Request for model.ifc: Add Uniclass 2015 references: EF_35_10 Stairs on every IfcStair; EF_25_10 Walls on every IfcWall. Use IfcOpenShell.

First a look at what the model holds.

```python
import ifcopenshell

model = ifcopenshell.open("model.ifc")
print(model.schema)
print("classifications:", [c.Name for c in model.by_type("IfcClassification")])
for ifc_class in ("IfcDoor", "IfcRoof", "IfcStair", "IfcWall", "IfcWindow"):
    print(ifc_class, len(model.by_type(ifc_class)))
```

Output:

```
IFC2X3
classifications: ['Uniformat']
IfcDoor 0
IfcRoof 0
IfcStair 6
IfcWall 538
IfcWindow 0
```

```python
import ifcopenshell
import ifcopenshell.api.classification

model = ifcopenshell.open("model.ifc")

# IFC2X3 requires Source and Edition and has no link from the project to the system.
system = model.create_entity("IfcClassification", Source="NBS", Edition="2015", Name="Uniclass 2015")

codes = {
    "IfcStair": ("EF_35_10", "Stairs"),
    "IfcWall": ("EF_25_10", "Walls"),
}
for ifc_class, (code, name) in codes.items():
    products = model.by_type(ifc_class)
    ifcopenshell.api.classification.add_reference(
        model, products=products, classification=system, identification=code, name=name
    )
    print(code, len(products))

model.write("model_updated.ifc")
```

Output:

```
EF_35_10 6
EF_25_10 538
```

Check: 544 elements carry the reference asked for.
